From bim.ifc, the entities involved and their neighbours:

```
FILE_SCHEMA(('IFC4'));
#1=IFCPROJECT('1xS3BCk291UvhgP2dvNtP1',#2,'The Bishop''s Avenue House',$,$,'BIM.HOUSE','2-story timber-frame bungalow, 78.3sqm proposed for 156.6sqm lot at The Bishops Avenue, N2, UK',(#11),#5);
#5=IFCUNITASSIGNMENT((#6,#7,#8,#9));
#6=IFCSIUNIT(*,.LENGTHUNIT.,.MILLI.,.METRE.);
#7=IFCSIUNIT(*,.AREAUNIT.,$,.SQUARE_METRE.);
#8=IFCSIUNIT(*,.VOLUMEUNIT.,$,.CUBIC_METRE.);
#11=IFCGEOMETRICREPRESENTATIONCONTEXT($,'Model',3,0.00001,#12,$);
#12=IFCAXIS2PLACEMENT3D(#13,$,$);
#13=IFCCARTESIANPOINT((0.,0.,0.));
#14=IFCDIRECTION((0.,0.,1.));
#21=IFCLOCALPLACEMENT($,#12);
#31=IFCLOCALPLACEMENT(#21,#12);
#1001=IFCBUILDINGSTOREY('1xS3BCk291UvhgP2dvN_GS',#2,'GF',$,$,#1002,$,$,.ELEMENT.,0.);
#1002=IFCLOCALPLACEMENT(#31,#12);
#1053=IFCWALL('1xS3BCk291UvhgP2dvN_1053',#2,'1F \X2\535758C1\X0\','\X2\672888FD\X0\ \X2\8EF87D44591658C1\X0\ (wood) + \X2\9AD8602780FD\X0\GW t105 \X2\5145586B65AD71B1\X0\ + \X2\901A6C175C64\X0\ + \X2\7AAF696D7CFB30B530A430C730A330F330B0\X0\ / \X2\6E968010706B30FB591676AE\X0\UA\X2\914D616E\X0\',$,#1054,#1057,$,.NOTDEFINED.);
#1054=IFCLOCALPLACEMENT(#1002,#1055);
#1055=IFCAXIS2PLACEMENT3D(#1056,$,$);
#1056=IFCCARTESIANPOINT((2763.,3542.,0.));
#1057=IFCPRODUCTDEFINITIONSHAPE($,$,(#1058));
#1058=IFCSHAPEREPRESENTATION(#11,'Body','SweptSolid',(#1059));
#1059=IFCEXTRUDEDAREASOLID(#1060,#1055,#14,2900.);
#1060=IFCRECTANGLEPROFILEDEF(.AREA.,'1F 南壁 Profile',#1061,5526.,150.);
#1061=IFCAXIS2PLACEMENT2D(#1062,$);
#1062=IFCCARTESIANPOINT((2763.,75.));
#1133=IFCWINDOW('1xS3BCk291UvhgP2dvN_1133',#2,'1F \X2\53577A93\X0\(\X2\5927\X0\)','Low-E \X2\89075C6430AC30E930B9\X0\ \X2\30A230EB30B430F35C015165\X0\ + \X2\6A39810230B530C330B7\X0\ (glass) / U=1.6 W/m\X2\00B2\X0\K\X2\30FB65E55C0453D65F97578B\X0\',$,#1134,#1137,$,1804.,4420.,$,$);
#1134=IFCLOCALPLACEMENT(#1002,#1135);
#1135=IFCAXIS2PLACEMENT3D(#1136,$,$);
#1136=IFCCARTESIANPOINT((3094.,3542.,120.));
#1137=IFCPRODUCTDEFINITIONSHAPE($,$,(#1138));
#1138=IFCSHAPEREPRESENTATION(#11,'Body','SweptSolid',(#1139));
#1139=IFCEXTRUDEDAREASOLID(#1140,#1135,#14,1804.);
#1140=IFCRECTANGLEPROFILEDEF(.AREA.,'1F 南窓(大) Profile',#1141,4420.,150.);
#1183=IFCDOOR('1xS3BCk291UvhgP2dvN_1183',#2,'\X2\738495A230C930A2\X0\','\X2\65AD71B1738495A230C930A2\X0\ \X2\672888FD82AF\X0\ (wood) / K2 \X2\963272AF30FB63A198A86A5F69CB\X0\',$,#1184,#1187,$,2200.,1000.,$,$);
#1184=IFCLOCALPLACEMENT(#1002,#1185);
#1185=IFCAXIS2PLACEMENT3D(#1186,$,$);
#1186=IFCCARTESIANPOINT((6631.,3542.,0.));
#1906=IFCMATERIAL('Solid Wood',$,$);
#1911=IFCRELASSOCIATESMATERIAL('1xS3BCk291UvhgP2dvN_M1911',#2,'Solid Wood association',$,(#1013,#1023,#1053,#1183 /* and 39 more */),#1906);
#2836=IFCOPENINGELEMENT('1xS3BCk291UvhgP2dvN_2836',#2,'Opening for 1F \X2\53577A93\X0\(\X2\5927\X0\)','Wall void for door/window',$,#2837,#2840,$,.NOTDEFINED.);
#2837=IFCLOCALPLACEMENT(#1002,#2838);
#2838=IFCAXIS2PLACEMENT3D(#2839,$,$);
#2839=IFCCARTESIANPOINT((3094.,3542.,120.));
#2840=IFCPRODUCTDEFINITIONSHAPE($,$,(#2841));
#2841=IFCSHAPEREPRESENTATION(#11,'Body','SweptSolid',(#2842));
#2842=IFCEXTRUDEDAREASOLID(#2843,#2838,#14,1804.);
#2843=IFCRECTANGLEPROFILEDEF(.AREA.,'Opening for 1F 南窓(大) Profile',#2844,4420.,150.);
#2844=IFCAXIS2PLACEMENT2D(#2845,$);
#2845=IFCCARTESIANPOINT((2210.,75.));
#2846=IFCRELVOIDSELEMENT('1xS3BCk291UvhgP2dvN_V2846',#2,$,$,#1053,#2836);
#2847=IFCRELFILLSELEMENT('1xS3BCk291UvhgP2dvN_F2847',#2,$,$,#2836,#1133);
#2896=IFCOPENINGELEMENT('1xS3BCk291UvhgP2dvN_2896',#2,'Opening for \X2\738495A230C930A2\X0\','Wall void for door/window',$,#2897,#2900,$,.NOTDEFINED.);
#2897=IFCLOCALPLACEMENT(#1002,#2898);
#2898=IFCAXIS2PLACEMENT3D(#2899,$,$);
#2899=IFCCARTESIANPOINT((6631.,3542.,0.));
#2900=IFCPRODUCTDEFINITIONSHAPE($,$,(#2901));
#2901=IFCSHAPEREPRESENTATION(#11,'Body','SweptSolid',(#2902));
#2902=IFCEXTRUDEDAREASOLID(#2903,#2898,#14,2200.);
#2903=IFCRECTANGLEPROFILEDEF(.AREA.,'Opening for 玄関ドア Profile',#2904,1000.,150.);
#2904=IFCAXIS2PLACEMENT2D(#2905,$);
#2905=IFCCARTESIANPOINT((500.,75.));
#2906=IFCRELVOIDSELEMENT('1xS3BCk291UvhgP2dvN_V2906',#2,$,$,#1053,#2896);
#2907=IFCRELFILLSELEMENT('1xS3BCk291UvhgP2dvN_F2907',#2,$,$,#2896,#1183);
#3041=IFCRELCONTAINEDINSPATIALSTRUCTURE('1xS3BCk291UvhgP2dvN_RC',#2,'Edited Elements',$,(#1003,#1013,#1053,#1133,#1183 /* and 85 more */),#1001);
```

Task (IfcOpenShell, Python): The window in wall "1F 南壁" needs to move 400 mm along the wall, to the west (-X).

```python
import ifcopenshell
import ifcopenshell.api.geometry
import ifcopenshell.util.placement

model = ifcopenshell.open("bim.ifc")

window = model.by_guid("1xS3BCk291UvhgP2dvN_1133")
opening = window.FillsVoids[0].RelatingOpeningElement
wall = opening.VoidsElements[0].RelatingBuildingElement

wall_matrix = ifcopenshell.util.placement.get_local_placement(wall.ObjectPlacement)
shift = wall_matrix[:3, 0] * -400.0
before = ifcopenshell.util.placement.get_local_placement(window.ObjectPlacement)[:3, 3].copy()

# The window is not placed relative to its opening, so move both.
for product in (opening, window):
    matrix = ifcopenshell.util.placement.get_local_placement(product.ObjectPlacement)
    matrix[:3, 3] += shift
    ifcopenshell.api.geometry.edit_object_placement(model, product=product, matrix=matrix, is_si=False)

after = ifcopenshell.util.placement.get_local_placement(window.ObjectPlacement)[:3, 3]
print("window moved by", (after - before).round(3) + 0.0)

model.write("bim-out.ifc")
```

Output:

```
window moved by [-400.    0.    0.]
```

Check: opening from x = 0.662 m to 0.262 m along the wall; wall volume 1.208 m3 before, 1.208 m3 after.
